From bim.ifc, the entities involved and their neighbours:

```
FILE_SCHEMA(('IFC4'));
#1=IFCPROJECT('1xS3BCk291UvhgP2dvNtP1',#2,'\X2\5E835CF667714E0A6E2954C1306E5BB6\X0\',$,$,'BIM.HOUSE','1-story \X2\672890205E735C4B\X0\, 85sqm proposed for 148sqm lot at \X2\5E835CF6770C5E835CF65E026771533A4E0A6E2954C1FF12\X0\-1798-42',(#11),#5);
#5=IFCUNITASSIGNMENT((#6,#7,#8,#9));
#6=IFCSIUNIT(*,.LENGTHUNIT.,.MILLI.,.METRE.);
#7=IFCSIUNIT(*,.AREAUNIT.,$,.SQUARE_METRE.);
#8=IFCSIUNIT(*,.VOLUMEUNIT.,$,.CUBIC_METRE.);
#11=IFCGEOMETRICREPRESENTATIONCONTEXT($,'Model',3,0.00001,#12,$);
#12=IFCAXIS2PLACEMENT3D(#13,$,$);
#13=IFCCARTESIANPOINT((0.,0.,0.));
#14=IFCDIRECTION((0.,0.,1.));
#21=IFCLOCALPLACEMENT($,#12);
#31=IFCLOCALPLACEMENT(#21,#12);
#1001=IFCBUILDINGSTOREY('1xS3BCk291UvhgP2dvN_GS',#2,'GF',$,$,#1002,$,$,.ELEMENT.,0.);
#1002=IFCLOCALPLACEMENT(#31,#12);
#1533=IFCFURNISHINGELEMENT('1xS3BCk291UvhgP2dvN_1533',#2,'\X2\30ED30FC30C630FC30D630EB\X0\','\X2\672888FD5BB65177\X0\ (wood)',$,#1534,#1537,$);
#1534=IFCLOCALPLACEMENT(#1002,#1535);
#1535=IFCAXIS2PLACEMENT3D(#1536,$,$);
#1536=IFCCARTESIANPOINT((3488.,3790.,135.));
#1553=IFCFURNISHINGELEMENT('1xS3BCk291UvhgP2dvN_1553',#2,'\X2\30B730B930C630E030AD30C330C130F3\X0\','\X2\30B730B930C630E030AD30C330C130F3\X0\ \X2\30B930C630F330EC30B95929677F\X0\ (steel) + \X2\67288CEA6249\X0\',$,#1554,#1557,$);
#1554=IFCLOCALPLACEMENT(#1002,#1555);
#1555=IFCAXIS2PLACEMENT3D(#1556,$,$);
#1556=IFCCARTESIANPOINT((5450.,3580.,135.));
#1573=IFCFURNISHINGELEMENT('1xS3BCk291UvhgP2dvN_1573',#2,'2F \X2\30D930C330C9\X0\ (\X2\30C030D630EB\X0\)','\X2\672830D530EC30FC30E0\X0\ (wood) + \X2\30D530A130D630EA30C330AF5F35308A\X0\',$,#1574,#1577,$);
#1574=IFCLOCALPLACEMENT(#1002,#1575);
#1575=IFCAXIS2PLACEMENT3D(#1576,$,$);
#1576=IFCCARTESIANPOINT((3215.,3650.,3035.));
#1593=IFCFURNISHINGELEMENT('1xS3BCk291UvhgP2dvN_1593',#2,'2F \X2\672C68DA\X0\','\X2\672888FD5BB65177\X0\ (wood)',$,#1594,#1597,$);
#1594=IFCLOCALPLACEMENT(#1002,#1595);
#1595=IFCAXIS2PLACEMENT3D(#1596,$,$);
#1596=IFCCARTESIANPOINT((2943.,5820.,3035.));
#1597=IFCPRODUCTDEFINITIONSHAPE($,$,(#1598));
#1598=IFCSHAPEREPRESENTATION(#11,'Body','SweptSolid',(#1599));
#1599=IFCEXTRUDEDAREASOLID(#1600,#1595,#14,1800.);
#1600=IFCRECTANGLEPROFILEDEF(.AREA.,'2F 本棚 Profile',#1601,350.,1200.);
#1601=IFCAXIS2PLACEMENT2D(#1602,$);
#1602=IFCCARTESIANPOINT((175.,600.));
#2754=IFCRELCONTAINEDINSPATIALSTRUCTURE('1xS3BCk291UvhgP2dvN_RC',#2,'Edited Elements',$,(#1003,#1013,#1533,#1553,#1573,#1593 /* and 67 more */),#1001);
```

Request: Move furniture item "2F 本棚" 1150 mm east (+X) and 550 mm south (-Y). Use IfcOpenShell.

```python
import ifcopenshell
import ifcopenshell.api.geometry
import ifcopenshell.util.placement
import ifcopenshell.util.unit

model = ifcopenshell.open("bim.ifc")
unit_scale = ifcopenshell.util.unit.calculate_unit_scale(model)

item = model.by_guid("1xS3BCk291UvhgP2dvN_1593")
matrix = ifcopenshell.util.placement.get_local_placement(item.ObjectPlacement)
matrix[0, 3] += 1.15 / unit_scale
matrix[1, 3] -= 0.55 / unit_scale
ifcopenshell.api.geometry.edit_object_placement(model, product=item, matrix=matrix, is_si=False)

print(ifcopenshell.util.placement.get_local_placement(item.ObjectPlacement).round(3) + 0.0)

model.write("bim_v2.ifc")
```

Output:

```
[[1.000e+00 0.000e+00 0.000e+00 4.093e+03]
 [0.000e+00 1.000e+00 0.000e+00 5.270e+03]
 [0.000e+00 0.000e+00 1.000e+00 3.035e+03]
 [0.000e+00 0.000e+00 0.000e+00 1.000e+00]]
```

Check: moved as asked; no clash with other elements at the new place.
